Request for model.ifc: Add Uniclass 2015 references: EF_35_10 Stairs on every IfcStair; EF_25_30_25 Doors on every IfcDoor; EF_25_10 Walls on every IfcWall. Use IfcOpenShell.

First a look at what the model holds.

```python
import ifcopenshell

model = ifcopenshell.open("model.ifc")
print(model.schema)
print("classifications:", [c.Name for c in model.by_type("IfcClassification")])
for ifc_class in ("IfcDoor", "IfcRoof", "IfcStair", "IfcWall", "IfcWindow"):
    print(ifc_class, len(model.by_type(ifc_class)))
```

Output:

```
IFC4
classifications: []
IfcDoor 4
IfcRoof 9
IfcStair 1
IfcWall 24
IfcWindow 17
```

```python
import ifcopenshell
import ifcopenshell.api.classification

model = ifcopenshell.open("model.ifc")

system = ifcopenshell.api.classification.add_classification(model, classification="Uniclass 2015")

codes = {
    "IfcStair": ("EF_35_10", "Stairs"),
    "IfcDoor": ("EF_25_30_25", "Doors"),
    "IfcWall": ("EF_25_10", "Walls"),
}
for ifc_class, (code, name) in codes.items():
    products = model.by_type(ifc_class)
    ifcopenshell.api.classification.add_reference(
        model, products=products, classification=system, identification=code, name=name
    )
    print(code, len(products))

model.write("model_edited.ifc")
```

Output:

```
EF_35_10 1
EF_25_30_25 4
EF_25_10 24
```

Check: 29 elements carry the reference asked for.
